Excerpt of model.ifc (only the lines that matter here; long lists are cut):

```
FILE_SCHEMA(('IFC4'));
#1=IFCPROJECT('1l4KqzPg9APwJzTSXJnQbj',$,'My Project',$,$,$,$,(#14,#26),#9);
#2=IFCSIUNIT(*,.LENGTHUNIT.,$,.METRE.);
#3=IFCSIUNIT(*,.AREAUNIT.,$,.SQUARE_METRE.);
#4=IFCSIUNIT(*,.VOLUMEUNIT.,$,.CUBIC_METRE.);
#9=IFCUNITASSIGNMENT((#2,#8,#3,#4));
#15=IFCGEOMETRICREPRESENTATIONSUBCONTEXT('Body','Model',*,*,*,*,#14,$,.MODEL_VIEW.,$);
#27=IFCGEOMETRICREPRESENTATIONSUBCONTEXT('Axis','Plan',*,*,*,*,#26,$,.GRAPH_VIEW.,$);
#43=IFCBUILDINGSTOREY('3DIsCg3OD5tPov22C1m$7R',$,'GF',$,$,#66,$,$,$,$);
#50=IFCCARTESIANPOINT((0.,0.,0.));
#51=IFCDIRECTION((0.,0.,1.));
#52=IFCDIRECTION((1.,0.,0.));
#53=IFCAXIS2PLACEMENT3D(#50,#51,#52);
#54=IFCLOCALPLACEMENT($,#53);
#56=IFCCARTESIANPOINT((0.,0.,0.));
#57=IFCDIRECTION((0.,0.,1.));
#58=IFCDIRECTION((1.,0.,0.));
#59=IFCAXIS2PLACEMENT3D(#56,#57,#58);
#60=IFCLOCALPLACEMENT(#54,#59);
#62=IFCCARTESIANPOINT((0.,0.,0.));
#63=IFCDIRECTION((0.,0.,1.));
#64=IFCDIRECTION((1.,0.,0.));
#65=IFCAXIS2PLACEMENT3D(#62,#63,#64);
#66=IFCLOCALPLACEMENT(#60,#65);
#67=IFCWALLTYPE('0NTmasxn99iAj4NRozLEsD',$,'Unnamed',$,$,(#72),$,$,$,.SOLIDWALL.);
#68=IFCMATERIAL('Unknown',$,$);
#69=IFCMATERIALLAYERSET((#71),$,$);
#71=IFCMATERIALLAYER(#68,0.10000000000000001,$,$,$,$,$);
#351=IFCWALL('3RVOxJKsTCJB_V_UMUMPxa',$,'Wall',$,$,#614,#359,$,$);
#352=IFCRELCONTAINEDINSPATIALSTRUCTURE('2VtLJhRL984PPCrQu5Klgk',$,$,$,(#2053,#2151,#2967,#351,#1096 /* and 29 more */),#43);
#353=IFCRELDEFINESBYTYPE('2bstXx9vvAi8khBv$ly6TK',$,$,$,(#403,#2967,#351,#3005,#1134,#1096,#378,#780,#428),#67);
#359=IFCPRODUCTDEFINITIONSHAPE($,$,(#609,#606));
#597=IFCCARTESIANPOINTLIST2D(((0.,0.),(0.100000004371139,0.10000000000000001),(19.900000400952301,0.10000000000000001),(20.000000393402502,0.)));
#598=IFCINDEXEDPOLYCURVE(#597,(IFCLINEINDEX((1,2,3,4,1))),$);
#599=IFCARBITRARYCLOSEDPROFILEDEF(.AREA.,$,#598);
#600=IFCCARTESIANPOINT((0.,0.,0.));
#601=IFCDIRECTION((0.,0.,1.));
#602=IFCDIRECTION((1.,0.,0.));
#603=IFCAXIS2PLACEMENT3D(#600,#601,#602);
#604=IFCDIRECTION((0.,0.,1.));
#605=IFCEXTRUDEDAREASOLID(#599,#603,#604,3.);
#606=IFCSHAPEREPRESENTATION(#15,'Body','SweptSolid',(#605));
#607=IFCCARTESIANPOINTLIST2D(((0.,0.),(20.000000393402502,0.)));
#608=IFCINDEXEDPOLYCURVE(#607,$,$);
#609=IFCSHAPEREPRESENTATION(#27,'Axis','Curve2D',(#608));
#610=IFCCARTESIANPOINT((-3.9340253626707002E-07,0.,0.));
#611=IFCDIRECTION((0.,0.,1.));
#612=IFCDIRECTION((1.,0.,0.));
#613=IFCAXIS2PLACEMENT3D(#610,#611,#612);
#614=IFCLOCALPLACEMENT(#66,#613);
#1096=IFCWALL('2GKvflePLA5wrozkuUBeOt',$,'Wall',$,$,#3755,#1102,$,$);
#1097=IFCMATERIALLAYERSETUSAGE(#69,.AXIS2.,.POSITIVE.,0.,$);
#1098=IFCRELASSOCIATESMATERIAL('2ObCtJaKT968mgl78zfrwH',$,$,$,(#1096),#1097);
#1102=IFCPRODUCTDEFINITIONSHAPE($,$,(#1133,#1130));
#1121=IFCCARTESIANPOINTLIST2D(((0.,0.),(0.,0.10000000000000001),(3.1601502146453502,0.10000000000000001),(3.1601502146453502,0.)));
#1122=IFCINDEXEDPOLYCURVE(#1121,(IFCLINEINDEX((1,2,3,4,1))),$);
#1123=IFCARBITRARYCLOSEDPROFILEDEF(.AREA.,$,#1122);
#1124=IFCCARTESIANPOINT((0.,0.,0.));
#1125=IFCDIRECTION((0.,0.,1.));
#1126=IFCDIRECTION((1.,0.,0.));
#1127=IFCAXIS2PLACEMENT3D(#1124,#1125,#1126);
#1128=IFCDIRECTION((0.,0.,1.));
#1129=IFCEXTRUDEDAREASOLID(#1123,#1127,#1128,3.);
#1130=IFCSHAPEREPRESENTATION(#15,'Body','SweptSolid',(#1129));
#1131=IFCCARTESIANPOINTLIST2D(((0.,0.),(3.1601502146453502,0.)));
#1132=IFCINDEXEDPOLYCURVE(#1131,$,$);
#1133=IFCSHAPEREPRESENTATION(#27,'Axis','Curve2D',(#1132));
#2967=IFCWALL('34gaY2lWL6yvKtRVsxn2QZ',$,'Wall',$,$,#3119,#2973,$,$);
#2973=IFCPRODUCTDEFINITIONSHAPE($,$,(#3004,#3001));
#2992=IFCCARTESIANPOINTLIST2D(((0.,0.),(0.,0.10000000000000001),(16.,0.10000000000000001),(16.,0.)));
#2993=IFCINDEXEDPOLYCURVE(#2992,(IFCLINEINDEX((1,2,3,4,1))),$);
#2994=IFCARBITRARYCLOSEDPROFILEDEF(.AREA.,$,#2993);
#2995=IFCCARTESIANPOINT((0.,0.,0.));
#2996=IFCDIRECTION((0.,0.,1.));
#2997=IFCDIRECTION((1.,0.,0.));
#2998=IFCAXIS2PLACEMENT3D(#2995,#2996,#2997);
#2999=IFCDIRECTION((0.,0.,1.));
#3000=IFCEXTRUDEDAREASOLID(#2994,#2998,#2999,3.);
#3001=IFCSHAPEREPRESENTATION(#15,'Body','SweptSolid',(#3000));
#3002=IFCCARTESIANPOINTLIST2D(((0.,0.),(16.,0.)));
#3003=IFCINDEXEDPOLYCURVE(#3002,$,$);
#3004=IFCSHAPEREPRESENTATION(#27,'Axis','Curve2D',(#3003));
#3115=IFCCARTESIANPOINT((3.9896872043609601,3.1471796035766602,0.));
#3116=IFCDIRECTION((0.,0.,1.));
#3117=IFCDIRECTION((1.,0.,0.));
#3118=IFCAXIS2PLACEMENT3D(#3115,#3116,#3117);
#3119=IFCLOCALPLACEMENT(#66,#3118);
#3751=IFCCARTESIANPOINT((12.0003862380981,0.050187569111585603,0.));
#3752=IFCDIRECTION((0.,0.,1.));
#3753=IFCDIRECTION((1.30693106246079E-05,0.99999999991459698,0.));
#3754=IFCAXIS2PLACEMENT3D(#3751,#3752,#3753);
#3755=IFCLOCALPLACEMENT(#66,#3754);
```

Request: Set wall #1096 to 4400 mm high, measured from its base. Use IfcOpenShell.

```python
import ifcopenshell
import ifcopenshell.geom
import ifcopenshell.util.representation
import ifcopenshell.util.shape

model = ifcopenshell.open("model.ifc")
settings = ifcopenshell.geom.settings()


def volume(element):
    """Net volume in cubic metres, openings subtracted."""
    shape = ifcopenshell.geom.create_shape(settings, element)
    return ifcopenshell.util.shape.get_volume(shape.geometry)


wall = model.by_guid("2GKvflePLA5wrozkuUBeOt")
before = volume(wall)

body = ifcopenshell.util.representation.get_representation(wall, "Model", "Body")
solid = body.Items[0]
old_height = solid.Depth
solid.Depth = 4.4
after = volume(wall)

print(f"height {old_height:g} -> {solid.Depth:g}, volume {before:.3f} -> {after:.3f} m3")

model.write("model_v2.ifc")
```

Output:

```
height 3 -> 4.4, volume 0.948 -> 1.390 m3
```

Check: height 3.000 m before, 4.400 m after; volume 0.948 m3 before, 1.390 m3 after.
